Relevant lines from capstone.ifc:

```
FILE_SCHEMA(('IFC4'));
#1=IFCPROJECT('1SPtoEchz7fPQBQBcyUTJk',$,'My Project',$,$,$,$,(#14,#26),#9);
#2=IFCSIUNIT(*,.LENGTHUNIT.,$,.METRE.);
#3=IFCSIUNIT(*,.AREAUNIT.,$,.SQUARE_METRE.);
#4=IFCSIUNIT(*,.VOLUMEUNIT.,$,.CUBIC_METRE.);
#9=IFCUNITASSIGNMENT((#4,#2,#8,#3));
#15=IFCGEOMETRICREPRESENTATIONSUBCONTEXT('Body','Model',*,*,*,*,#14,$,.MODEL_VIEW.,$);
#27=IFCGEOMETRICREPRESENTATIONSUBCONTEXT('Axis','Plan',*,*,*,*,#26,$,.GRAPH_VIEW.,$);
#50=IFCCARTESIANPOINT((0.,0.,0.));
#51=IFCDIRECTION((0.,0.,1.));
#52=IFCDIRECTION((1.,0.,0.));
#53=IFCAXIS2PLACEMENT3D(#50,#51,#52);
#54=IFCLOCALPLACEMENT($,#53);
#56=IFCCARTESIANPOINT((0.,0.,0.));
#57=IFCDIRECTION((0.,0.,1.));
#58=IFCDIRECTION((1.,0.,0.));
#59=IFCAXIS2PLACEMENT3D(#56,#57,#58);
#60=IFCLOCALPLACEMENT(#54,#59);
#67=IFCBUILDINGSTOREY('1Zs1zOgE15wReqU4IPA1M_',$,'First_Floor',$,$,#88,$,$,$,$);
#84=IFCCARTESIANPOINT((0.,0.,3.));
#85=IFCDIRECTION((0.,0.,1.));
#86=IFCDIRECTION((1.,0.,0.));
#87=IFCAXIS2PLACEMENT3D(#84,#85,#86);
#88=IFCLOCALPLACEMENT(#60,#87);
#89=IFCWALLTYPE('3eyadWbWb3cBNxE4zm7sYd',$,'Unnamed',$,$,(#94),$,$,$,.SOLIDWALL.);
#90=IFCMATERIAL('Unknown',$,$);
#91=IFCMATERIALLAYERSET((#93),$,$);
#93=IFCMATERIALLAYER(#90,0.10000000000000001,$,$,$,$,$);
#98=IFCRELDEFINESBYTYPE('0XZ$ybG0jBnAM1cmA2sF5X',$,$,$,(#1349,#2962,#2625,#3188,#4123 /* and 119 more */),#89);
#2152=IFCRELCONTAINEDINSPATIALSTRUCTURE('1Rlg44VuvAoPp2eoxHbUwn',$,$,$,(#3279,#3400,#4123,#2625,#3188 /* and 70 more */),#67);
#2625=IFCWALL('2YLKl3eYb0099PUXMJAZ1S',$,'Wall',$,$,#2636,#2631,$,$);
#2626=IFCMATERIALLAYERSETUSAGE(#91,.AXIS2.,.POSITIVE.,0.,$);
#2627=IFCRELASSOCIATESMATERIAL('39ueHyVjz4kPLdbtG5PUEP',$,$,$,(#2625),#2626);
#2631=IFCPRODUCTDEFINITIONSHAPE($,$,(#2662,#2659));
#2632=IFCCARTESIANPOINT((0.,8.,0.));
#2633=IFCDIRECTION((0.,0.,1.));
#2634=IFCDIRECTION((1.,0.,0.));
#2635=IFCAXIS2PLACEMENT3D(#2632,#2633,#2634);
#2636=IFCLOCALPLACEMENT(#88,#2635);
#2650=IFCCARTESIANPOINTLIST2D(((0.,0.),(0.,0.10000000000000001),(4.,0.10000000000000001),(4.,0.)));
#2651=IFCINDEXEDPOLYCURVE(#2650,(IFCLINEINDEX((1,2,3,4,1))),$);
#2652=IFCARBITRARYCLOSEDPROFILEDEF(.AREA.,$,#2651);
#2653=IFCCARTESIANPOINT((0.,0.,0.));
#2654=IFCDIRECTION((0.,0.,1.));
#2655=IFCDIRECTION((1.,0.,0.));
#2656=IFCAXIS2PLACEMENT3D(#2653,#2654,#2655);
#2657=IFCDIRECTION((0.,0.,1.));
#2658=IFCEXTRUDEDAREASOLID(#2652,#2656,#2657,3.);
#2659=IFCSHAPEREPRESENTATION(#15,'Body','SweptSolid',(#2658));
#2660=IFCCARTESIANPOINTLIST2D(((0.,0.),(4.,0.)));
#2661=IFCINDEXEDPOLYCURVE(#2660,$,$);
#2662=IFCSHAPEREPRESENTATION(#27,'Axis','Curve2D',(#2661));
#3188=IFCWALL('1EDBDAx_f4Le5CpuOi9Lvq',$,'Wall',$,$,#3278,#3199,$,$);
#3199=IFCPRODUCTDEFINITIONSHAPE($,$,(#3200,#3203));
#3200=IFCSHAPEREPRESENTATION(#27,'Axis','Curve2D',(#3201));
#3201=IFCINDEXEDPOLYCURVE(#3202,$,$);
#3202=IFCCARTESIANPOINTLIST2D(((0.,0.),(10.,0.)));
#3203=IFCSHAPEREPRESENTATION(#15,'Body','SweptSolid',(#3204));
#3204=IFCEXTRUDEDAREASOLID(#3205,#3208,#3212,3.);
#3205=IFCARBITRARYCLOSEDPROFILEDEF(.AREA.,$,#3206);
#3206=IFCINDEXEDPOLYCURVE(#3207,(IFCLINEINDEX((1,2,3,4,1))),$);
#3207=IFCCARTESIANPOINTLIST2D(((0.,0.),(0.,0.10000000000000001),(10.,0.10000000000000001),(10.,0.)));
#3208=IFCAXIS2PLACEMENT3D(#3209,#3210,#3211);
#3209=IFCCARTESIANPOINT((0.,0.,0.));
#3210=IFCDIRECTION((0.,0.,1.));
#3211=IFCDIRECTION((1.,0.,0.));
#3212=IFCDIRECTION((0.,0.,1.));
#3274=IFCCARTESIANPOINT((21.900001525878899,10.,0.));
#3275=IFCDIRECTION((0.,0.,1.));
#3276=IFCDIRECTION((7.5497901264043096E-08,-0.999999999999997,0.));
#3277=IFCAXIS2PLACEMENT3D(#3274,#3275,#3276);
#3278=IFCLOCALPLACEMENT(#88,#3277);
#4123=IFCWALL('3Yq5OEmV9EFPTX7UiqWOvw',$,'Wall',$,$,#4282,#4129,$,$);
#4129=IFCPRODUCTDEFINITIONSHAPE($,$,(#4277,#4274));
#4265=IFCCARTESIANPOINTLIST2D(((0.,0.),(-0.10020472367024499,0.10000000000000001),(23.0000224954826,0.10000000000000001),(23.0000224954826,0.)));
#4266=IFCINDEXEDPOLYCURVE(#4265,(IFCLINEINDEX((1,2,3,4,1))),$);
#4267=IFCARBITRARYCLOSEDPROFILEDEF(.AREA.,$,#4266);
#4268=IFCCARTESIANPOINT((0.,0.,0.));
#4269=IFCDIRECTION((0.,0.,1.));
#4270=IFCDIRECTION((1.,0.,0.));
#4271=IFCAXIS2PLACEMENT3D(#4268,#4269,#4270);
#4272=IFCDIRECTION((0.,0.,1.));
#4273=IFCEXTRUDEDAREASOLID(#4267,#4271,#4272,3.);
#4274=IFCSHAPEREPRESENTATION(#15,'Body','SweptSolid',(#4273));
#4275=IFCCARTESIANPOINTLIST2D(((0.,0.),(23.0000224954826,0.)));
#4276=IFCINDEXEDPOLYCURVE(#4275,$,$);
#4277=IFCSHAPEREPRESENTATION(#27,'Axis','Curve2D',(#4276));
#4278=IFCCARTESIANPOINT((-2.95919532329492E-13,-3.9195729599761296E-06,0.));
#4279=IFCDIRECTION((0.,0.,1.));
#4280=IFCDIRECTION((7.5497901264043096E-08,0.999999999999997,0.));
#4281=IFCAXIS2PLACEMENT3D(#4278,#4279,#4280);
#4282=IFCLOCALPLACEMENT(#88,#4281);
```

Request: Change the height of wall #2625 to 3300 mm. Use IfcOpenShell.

```python
import ifcopenshell
import ifcopenshell.geom
import ifcopenshell.util.representation
import ifcopenshell.util.shape

model = ifcopenshell.open("capstone.ifc")
settings = ifcopenshell.geom.settings()


def volume(element):
    """Net volume in cubic metres, openings subtracted."""
    shape = ifcopenshell.geom.create_shape(settings, element)
    return ifcopenshell.util.shape.get_volume(shape.geometry)


wall = model.by_guid("2YLKl3eYb0099PUXMJAZ1S")
before = volume(wall)

body = ifcopenshell.util.representation.get_representation(wall, "Model", "Body")
solid = body.Items[0]
old_height = solid.Depth
solid.Depth = 3.3
after = volume(wall)

print(f"height {old_height:g} -> {solid.Depth:g}, volume {before:.3f} -> {after:.3f} m3")

model.write("capstone_updated.ifc")
```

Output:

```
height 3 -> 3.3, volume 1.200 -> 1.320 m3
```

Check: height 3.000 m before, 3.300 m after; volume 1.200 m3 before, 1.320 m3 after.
